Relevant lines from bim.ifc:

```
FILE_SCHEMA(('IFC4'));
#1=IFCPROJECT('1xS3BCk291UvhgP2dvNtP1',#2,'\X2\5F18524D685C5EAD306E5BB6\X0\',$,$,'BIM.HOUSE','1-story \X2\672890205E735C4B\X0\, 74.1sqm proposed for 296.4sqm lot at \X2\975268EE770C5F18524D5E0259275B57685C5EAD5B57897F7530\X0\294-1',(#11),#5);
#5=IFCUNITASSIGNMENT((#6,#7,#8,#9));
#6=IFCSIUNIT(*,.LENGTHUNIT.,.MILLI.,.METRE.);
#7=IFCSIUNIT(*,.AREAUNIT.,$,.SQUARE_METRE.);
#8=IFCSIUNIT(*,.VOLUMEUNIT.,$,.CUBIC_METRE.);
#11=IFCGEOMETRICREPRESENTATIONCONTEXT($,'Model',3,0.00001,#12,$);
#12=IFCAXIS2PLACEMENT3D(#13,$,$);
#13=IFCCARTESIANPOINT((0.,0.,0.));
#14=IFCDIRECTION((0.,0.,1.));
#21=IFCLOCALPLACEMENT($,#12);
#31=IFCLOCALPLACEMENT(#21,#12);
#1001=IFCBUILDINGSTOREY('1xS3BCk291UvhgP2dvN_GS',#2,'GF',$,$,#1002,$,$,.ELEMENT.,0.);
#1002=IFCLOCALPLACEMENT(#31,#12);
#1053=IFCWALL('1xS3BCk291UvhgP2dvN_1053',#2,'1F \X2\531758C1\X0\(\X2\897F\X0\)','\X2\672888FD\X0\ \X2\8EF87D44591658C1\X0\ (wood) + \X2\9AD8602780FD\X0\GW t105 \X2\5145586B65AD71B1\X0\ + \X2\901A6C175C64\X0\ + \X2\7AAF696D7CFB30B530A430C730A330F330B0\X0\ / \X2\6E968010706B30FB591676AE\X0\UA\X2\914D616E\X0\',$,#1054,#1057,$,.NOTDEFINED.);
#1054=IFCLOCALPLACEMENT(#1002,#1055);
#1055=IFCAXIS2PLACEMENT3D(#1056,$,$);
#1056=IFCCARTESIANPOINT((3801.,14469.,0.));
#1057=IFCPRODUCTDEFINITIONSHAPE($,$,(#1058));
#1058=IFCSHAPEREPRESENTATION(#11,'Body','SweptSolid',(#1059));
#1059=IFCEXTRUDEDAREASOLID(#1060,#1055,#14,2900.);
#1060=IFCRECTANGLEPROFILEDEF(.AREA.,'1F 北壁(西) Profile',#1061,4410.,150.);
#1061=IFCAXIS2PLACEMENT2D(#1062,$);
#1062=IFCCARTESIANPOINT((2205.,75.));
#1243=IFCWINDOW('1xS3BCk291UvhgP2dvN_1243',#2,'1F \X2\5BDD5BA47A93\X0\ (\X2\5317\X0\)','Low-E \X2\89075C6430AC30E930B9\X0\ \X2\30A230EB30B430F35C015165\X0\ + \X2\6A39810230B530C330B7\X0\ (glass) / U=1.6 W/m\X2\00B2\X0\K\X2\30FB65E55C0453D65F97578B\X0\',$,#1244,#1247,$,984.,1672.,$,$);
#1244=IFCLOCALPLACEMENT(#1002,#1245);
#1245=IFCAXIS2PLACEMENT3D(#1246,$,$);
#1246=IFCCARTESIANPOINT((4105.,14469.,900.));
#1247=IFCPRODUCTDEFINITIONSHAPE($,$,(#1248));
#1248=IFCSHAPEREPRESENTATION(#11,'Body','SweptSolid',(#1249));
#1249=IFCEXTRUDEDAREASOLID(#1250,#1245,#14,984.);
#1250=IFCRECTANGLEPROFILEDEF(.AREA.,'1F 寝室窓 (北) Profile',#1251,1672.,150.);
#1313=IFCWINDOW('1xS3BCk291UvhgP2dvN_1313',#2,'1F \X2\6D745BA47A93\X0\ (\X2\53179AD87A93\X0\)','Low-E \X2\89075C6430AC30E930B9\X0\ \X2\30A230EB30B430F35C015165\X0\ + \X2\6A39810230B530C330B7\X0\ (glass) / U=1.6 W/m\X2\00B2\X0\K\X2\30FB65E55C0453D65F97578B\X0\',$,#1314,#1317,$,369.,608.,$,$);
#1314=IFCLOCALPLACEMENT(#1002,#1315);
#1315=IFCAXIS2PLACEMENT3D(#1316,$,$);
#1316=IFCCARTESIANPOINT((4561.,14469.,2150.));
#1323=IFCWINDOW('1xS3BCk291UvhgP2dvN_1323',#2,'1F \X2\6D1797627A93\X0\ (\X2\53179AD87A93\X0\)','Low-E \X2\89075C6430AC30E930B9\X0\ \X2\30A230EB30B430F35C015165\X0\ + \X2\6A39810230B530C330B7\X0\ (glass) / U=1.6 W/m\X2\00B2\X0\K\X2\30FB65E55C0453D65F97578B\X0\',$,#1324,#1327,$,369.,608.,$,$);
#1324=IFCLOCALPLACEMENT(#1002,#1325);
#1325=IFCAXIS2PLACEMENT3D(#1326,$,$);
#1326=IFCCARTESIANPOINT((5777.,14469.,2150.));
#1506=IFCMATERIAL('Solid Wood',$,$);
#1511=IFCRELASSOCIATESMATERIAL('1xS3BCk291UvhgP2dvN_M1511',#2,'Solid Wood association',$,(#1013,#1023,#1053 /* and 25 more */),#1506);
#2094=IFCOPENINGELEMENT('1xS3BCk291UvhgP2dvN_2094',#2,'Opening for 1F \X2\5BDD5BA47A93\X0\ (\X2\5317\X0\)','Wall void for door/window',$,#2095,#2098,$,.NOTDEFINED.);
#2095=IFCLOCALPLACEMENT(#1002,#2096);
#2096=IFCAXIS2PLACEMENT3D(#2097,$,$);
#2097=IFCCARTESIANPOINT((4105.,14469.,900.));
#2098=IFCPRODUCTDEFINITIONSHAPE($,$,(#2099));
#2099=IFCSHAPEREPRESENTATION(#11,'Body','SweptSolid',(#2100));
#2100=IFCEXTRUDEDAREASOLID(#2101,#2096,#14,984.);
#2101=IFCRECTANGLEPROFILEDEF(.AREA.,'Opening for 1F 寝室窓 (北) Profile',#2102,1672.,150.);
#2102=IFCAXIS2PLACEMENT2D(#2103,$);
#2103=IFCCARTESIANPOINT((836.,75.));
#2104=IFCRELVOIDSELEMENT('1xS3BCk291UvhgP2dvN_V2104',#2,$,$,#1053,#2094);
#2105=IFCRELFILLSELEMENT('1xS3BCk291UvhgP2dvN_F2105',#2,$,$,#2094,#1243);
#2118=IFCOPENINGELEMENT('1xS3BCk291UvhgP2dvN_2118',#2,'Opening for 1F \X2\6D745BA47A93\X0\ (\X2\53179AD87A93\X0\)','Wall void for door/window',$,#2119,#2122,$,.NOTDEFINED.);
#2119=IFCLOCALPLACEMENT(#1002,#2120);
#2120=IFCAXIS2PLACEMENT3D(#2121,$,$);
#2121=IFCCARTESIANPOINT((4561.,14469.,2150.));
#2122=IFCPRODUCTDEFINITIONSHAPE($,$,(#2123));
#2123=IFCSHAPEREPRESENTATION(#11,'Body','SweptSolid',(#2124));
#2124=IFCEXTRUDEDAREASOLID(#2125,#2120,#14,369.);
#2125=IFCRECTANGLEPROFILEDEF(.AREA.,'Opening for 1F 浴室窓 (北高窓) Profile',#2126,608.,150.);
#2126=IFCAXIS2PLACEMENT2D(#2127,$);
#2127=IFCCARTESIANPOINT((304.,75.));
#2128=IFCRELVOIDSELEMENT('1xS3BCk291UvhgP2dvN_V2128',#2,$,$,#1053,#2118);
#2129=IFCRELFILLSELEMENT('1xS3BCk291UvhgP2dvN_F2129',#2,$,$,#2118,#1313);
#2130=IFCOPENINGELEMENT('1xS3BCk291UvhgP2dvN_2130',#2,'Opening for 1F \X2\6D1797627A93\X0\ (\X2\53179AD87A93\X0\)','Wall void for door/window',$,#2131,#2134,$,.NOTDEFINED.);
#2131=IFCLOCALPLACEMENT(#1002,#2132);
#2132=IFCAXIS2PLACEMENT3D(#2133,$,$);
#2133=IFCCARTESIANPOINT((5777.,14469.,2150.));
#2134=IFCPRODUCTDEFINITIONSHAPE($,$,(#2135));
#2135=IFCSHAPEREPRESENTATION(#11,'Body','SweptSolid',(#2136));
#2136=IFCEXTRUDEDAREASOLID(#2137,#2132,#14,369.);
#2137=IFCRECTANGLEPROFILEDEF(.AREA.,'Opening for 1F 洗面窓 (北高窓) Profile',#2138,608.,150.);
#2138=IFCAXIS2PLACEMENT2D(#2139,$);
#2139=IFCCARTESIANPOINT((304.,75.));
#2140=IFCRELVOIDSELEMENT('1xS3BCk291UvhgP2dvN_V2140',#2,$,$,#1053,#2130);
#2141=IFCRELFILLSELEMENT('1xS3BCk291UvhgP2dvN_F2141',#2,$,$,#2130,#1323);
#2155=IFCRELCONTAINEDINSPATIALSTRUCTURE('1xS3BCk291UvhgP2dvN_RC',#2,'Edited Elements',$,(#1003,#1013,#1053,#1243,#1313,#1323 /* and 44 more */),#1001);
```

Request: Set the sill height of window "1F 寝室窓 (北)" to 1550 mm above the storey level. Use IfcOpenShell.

```python
import numpy as np
import ifcopenshell
import ifcopenshell.api.geometry
import ifcopenshell.geom
import ifcopenshell.util.element
import ifcopenshell.util.placement
import ifcopenshell.util.shape
import ifcopenshell.util.unit

model = ifcopenshell.open("bim.ifc")
unit_scale = ifcopenshell.util.unit.calculate_unit_scale(model)

window = model.by_id(1243)
opening = window.FillsVoids[0].RelatingOpeningElement
storey = ifcopenshell.util.element.get_container(window, ifc_class="IfcBuildingStorey")
level = ifcopenshell.util.placement.get_local_placement(storey.ObjectPlacement)[2, 3]

# The opening's origin need not be at the sill, so measure its lowest point.
shape = ifcopenshell.geom.create_shape(ifcopenshell.geom.settings(), opening)
bottom = ifcopenshell.util.shape.get_shape_bottom_elevation(shape, shape.geometry) / unit_scale
dz = level + 1.55 / unit_scale - bottom

shift = np.array([0.0, 0.0, dz])
# The window is not placed relative to its opening, so move both.
for product in (opening, window):
    matrix = ifcopenshell.util.placement.get_local_placement(product.ObjectPlacement)
    matrix[:3, 3] += shift
    ifcopenshell.api.geometry.edit_object_placement(model, product=product, matrix=matrix, is_si=False)

print(f"moved by {dz * unit_scale:+.3f} m")

model.write("bim_rev.ifc")
```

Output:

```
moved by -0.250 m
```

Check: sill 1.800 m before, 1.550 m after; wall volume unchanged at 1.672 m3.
